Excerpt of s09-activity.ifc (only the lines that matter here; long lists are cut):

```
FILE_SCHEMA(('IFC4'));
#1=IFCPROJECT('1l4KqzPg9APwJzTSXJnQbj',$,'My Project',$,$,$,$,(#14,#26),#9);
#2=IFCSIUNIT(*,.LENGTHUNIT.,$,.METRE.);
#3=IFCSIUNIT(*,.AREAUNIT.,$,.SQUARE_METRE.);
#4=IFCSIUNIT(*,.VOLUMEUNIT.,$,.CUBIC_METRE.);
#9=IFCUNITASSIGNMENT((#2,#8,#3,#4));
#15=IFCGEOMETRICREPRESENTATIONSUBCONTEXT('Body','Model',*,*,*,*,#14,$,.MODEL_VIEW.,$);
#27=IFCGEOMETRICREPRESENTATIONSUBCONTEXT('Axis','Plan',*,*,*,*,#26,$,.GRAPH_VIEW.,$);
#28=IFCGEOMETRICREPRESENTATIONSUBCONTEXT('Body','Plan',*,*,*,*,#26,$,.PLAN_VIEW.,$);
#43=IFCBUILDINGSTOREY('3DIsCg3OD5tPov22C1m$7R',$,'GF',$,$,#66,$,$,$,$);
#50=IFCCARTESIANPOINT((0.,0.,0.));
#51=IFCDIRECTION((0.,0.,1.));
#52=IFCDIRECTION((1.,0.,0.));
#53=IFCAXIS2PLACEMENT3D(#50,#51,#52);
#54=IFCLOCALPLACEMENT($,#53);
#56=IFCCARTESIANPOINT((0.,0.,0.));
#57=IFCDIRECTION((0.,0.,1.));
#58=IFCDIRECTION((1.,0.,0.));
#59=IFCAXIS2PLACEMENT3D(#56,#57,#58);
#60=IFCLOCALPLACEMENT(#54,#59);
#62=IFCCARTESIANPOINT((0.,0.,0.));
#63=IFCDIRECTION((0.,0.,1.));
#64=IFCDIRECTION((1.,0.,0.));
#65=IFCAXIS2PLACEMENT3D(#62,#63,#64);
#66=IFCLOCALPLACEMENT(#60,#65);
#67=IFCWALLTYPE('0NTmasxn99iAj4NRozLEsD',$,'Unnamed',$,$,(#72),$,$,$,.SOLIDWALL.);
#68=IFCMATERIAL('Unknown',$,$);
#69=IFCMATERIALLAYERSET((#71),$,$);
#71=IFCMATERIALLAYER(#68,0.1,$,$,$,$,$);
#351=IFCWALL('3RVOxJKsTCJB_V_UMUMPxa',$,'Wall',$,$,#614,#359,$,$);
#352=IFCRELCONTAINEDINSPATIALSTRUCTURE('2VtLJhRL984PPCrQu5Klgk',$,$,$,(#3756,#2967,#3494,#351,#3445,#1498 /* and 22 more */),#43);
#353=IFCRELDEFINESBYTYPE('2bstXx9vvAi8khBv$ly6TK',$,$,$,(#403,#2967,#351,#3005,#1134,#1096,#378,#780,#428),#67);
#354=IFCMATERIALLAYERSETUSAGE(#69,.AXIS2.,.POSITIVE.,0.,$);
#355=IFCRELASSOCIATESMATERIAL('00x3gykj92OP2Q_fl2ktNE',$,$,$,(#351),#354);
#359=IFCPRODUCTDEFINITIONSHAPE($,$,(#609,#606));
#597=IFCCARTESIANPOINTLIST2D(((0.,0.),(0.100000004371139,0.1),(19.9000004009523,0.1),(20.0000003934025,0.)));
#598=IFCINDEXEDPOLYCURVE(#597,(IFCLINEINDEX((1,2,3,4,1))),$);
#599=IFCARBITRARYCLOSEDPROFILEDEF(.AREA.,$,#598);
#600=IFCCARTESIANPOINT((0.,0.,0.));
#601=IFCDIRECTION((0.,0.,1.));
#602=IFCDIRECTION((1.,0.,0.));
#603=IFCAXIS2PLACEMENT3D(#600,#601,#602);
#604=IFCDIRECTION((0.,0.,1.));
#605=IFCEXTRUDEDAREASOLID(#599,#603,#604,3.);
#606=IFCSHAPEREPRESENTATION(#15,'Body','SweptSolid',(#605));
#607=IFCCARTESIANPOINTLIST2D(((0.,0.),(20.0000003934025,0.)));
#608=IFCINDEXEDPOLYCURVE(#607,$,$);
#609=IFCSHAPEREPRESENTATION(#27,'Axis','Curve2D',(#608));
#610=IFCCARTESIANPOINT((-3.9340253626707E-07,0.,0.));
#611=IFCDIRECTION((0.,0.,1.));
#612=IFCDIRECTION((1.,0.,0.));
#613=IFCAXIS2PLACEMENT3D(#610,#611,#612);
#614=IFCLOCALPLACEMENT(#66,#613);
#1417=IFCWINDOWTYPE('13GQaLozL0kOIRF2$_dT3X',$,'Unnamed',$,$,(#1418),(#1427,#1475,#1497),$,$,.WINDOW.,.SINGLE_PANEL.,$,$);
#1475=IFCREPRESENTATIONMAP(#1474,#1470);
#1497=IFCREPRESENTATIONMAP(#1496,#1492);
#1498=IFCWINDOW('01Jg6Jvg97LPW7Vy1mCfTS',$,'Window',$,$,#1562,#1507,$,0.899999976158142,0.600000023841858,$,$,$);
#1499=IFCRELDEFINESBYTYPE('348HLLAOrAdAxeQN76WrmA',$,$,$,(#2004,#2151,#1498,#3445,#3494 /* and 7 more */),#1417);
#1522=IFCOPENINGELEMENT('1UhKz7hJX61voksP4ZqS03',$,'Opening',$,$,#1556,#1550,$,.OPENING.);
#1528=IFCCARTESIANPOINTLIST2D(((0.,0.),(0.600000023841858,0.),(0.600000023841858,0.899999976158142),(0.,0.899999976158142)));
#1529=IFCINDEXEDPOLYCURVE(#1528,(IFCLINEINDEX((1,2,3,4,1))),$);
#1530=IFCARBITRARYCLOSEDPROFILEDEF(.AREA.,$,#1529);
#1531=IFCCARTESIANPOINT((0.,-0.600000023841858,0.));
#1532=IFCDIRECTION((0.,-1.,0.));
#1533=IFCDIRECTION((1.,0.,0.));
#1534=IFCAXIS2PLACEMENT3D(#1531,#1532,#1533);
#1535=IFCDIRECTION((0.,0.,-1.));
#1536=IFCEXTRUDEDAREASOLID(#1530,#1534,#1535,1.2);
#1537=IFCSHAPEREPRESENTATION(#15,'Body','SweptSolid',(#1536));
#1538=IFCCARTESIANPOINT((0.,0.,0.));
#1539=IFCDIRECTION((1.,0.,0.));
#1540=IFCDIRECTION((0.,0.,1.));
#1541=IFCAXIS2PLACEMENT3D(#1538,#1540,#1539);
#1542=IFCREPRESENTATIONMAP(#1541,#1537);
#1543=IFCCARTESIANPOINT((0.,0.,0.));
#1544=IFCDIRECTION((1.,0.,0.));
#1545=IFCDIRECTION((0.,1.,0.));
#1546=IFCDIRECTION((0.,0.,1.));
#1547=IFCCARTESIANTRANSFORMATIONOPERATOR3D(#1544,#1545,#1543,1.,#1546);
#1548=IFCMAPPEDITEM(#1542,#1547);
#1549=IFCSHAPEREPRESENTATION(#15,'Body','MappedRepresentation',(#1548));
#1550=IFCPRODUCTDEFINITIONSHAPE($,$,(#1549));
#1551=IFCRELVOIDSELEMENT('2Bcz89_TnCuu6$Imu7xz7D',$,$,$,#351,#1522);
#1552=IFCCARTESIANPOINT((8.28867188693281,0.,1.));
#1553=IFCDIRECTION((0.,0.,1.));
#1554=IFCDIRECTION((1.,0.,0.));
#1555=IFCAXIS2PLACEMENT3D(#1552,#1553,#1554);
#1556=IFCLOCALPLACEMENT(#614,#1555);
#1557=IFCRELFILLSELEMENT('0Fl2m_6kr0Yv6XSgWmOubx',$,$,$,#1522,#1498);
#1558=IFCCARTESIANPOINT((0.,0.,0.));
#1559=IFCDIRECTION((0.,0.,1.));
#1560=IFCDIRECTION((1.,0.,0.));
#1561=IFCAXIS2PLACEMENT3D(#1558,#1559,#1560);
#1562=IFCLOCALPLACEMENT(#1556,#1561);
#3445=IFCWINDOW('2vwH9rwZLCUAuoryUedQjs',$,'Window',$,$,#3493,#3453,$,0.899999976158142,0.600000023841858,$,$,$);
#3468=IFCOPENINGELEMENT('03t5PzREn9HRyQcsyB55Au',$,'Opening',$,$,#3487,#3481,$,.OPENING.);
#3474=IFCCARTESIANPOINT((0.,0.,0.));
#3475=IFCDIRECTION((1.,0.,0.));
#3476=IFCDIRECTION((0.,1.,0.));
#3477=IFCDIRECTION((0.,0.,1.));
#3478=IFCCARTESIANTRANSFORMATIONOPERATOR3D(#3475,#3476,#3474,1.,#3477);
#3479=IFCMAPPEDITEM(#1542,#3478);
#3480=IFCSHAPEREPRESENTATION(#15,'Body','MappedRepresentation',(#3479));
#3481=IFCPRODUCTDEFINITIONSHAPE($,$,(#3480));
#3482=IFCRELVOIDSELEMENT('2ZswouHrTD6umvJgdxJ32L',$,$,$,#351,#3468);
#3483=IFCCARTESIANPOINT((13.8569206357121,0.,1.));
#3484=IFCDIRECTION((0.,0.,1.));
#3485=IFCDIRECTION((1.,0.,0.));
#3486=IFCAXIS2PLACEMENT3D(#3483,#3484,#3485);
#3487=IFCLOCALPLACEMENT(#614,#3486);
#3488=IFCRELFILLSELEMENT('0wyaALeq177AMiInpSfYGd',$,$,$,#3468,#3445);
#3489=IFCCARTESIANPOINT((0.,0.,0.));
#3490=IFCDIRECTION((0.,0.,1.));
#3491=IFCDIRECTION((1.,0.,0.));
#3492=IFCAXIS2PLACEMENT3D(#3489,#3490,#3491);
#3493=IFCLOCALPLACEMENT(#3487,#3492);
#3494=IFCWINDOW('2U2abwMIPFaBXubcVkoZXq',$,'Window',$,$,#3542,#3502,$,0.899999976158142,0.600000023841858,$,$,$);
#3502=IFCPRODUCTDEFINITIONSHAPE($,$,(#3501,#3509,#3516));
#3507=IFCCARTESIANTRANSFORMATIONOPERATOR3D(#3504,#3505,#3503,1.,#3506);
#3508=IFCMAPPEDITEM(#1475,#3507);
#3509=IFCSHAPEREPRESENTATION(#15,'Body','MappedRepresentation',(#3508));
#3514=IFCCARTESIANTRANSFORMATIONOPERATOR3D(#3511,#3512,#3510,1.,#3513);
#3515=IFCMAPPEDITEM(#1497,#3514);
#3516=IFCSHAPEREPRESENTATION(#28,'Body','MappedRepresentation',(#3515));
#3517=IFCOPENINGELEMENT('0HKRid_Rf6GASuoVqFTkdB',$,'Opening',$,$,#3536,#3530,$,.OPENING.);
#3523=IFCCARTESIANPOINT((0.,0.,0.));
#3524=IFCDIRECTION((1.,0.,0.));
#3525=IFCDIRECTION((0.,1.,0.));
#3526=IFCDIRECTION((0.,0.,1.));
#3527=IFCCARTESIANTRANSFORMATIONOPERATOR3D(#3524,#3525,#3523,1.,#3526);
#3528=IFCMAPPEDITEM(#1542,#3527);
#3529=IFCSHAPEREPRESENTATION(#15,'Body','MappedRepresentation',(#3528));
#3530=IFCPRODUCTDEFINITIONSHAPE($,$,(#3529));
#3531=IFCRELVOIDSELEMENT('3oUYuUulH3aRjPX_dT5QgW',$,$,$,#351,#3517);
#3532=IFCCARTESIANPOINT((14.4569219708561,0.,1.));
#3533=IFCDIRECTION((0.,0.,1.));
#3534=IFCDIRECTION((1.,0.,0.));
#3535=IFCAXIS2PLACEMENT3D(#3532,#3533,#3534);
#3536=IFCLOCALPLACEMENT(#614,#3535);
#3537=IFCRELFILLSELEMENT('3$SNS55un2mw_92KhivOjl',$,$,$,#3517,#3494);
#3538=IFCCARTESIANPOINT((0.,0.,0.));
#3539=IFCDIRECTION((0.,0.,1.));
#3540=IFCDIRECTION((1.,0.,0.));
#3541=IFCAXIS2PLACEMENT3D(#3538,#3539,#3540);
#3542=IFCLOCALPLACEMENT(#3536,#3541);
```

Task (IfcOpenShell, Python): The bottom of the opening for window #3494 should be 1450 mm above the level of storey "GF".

```python
import numpy as np
import ifcopenshell
import ifcopenshell.api.geometry
import ifcopenshell.geom
import ifcopenshell.util.element
import ifcopenshell.util.placement
import ifcopenshell.util.shape
import ifcopenshell.util.unit

model = ifcopenshell.open("s09-activity.ifc")
unit_scale = ifcopenshell.util.unit.calculate_unit_scale(model)

window = model.by_guid("2U2abwMIPFaBXubcVkoZXq")
opening = window.FillsVoids[0].RelatingOpeningElement
storey = ifcopenshell.util.element.get_container(window, ifc_class="IfcBuildingStorey")
level = ifcopenshell.util.placement.get_local_placement(storey.ObjectPlacement)[2, 3]

# The opening's origin need not be at the sill, so measure its lowest point.
shape = ifcopenshell.geom.create_shape(ifcopenshell.geom.settings(), opening)
bottom = ifcopenshell.util.shape.get_shape_bottom_elevation(shape, shape.geometry) / unit_scale
dz = level + 1.45 / unit_scale - bottom

shift = np.array([0.0, 0.0, dz])
# The window is placed relative to its opening, so it follows when the opening moves.
matrix = ifcopenshell.util.placement.get_local_placement(opening.ObjectPlacement)
matrix[:3, 3] += shift
ifcopenshell.api.geometry.edit_object_placement(
    model, product=opening, matrix=matrix, is_si=False, should_transform_children=True
)

print(f"moved by {dz * unit_scale:+.3f} m")

model.write("s09-activity_rev.ifc")
```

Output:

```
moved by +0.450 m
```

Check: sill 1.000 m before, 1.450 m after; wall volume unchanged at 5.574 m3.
